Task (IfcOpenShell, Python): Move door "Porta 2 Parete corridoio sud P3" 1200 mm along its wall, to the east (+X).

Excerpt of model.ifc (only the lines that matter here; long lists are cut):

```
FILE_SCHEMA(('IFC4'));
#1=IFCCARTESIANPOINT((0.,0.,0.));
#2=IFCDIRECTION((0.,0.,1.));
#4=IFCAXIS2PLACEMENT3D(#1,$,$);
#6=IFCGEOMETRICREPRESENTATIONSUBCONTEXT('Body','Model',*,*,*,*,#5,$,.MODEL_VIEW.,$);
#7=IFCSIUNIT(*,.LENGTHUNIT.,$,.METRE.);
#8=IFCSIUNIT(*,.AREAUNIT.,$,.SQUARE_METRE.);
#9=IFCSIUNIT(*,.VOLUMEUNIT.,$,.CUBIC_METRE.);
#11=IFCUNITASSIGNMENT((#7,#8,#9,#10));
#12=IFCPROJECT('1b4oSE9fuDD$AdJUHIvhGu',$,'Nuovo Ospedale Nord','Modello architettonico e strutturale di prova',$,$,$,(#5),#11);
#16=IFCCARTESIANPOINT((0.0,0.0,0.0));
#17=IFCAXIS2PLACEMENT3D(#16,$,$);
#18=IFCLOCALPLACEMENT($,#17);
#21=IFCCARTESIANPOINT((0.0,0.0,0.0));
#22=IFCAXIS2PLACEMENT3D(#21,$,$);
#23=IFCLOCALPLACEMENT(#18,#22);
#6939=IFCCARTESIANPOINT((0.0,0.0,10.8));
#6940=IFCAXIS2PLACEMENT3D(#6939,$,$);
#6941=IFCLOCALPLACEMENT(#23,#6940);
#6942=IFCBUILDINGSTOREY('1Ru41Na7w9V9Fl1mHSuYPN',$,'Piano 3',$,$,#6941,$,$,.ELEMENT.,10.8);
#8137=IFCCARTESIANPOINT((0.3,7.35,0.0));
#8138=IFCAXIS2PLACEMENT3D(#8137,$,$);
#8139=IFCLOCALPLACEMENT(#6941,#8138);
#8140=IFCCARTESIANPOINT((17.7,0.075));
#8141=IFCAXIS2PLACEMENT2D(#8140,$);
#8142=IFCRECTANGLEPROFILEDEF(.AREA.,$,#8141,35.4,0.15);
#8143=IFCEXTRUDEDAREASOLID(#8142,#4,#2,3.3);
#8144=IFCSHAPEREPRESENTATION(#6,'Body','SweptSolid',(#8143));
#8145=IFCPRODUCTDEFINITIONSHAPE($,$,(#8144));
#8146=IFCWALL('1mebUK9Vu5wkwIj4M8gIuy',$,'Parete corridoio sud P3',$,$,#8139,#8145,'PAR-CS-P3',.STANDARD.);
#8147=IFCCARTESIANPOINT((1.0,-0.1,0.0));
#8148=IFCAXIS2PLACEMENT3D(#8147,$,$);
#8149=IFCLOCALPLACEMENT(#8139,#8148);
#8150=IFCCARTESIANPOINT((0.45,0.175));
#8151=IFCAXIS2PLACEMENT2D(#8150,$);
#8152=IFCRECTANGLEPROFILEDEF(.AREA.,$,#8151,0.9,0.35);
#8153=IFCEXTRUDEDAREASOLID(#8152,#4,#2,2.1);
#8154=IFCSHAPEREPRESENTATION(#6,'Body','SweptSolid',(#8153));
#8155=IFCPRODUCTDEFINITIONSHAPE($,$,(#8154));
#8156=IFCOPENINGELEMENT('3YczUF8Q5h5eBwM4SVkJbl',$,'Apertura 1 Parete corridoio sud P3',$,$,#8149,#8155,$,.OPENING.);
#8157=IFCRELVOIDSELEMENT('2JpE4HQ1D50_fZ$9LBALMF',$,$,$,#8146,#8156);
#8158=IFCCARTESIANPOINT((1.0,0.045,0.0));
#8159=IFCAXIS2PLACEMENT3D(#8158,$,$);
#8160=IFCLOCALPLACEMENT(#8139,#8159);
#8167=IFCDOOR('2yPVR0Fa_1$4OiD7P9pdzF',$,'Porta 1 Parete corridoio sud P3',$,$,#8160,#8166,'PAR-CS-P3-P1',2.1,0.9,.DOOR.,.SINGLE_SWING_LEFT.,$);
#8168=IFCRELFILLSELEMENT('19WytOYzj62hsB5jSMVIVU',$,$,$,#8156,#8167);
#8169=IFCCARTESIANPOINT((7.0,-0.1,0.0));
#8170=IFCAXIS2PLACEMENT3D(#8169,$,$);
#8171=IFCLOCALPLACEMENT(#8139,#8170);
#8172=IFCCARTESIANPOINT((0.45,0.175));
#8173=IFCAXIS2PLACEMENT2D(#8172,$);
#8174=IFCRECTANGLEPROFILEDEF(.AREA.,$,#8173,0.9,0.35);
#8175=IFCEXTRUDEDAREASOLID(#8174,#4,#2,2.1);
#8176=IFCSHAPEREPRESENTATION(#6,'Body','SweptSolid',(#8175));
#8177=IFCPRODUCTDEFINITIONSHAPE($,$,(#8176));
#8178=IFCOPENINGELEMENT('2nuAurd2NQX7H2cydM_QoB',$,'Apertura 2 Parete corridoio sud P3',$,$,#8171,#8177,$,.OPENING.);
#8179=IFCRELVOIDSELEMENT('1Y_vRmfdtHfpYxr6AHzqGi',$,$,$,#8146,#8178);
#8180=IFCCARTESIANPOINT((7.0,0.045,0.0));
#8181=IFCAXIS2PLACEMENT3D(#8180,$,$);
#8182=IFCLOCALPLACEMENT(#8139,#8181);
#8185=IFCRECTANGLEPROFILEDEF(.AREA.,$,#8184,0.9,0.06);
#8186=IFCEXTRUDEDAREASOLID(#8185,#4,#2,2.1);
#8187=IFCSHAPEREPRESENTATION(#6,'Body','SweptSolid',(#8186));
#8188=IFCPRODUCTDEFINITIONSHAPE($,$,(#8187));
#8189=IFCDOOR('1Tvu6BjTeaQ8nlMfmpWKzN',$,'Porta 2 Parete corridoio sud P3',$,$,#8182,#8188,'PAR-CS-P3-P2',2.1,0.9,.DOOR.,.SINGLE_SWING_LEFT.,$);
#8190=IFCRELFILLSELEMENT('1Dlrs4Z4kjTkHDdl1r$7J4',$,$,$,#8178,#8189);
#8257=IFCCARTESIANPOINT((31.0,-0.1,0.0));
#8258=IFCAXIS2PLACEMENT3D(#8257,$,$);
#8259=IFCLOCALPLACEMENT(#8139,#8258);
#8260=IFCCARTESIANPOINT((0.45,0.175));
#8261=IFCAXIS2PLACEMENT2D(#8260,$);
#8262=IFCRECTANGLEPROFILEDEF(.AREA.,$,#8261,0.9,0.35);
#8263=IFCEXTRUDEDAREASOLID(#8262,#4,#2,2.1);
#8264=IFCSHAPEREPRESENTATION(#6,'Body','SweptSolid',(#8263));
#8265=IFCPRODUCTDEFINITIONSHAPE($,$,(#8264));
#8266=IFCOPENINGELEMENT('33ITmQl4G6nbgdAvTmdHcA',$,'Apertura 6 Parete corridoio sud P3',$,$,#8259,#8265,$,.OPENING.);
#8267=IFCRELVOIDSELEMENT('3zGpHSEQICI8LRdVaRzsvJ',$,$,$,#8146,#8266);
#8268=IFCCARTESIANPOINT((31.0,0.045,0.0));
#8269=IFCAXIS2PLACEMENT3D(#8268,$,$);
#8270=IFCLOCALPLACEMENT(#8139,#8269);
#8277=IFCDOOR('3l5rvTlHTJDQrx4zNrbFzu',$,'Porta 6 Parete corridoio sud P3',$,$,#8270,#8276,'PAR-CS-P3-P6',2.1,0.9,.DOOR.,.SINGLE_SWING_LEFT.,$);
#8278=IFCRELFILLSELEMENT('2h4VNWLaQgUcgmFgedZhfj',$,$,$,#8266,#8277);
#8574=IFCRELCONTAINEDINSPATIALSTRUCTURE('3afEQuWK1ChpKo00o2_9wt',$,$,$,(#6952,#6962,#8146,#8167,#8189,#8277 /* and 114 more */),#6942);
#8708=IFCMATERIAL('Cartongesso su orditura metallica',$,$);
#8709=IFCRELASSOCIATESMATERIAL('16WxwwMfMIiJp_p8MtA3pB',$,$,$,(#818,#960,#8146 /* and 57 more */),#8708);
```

```python
import ifcopenshell
import ifcopenshell.api.geometry
import ifcopenshell.util.placement

model = ifcopenshell.open("model.ifc")

door = model.by_id(8189)
opening = door.FillsVoids[0].RelatingOpeningElement
wall = opening.VoidsElements[0].RelatingBuildingElement

wall_matrix = ifcopenshell.util.placement.get_local_placement(wall.ObjectPlacement)
shift = wall_matrix[:3, 0] * 1.2
before = ifcopenshell.util.placement.get_local_placement(door.ObjectPlacement)[:3, 3].copy()

# The door is not placed relative to its opening, so move both.
for product in (opening, door):
    matrix = ifcopenshell.util.placement.get_local_placement(product.ObjectPlacement)
    matrix[:3, 3] += shift
    ifcopenshell.api.geometry.edit_object_placement(model, product=product, matrix=matrix, is_si=False)

after = ifcopenshell.util.placement.get_local_placement(door.ObjectPlacement)[:3, 3]
print("door moved by", (after - before).round(3) + 0.0)

model.write("model-out.ifc")
```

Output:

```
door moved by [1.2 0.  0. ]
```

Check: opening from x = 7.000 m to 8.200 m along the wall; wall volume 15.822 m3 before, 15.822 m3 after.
